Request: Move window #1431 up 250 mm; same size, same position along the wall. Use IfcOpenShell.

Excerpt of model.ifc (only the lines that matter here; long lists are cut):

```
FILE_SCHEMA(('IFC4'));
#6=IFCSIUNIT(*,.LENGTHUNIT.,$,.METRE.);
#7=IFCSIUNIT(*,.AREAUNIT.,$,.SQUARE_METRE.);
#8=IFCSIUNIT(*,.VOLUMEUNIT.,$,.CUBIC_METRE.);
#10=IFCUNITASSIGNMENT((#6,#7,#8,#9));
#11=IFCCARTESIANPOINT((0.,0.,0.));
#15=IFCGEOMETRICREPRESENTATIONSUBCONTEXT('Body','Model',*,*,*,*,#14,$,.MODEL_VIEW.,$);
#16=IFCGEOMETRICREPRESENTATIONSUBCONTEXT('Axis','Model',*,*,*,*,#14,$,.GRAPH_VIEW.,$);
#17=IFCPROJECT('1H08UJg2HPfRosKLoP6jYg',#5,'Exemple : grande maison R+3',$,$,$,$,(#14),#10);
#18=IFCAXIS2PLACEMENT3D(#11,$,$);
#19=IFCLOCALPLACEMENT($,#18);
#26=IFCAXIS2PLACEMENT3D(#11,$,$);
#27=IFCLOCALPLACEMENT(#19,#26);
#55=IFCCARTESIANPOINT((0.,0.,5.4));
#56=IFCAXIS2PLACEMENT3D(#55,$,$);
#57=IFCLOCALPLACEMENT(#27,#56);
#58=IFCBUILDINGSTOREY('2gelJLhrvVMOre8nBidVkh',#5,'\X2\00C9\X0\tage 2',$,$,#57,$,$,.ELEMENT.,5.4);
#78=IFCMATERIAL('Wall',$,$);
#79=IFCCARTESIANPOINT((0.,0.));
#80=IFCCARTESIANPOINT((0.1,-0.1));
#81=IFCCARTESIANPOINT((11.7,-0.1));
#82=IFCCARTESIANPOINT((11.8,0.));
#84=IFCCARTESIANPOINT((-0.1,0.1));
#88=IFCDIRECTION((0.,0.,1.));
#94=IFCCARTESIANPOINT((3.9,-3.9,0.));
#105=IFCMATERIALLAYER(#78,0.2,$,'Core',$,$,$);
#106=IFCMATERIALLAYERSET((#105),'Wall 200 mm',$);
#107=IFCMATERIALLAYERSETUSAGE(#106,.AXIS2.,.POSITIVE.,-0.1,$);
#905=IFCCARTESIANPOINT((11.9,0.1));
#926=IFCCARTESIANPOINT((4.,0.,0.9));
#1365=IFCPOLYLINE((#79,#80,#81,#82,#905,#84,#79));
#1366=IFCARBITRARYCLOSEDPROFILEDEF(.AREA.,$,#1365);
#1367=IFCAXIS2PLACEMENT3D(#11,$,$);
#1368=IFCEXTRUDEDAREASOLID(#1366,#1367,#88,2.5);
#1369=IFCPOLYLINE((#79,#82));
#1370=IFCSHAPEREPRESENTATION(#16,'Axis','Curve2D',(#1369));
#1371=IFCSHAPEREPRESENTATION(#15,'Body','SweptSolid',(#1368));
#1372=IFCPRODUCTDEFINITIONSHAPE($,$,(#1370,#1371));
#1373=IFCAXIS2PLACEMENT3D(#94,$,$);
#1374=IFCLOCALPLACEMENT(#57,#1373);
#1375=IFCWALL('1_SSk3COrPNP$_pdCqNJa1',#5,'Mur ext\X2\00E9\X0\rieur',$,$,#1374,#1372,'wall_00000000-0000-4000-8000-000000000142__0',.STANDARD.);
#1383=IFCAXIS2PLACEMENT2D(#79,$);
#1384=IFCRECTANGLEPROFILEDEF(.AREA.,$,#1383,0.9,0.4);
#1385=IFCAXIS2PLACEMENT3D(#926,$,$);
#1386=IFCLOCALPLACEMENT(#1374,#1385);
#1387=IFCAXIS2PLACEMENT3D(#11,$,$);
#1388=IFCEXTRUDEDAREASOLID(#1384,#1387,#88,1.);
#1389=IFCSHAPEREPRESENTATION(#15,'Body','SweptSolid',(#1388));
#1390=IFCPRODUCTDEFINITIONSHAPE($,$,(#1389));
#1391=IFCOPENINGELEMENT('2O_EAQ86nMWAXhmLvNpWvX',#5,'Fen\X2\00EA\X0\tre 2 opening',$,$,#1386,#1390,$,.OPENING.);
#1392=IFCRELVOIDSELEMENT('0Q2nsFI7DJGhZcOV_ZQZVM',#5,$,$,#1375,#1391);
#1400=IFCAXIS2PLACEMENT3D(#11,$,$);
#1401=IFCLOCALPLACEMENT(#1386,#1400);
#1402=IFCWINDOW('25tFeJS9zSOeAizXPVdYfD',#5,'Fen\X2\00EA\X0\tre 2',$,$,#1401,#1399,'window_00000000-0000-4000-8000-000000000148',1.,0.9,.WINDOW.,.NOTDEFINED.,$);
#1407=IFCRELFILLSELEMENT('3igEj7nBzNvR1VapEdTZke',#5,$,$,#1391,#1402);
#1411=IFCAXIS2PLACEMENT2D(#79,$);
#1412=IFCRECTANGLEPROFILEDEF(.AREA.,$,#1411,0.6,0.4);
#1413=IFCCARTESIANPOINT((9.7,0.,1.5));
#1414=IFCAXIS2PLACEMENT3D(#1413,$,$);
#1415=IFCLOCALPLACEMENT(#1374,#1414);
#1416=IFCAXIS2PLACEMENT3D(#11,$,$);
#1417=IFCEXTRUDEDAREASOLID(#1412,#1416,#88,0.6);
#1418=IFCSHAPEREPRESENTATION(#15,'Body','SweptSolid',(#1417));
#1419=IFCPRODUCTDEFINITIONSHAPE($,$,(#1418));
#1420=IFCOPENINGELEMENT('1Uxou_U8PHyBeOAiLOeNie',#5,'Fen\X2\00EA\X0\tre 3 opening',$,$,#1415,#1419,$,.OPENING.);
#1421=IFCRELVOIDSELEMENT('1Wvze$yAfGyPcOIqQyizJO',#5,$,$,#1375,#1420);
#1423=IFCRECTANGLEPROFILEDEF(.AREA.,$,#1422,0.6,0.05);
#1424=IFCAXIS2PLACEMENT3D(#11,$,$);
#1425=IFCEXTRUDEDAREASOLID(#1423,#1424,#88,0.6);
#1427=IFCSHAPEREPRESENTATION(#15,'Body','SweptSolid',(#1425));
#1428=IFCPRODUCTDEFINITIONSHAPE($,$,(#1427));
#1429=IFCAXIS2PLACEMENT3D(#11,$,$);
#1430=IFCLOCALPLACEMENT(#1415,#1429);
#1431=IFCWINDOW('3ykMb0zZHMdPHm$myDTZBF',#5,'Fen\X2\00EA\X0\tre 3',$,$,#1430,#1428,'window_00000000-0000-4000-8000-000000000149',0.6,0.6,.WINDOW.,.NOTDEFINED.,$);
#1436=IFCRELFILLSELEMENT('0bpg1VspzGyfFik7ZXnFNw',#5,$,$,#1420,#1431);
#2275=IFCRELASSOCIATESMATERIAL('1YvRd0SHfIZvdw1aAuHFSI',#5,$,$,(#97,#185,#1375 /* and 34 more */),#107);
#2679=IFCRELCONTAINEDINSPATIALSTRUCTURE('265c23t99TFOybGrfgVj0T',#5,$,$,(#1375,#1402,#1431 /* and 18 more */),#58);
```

```python
import numpy as np
import ifcopenshell
import ifcopenshell.api.geometry
import ifcopenshell.util.placement
import ifcopenshell.util.unit

model = ifcopenshell.open("model.ifc")
unit_scale = ifcopenshell.util.unit.calculate_unit_scale(model)

window = model.by_guid("3ykMb0zZHMdPHm$myDTZBF")
opening = window.FillsVoids[0].RelatingOpeningElement
dz = 0.25 / unit_scale

shift = np.array([0.0, 0.0, dz])
# The window is placed relative to its opening, so it follows when the opening moves.
matrix = ifcopenshell.util.placement.get_local_placement(opening.ObjectPlacement)
matrix[:3, 3] += shift
ifcopenshell.api.geometry.edit_object_placement(
    model, product=opening, matrix=matrix, is_si=False, should_transform_children=True
)

print(f"moved by {dz * unit_scale:+.3f} m")

model.write("model_rev.ifc")
```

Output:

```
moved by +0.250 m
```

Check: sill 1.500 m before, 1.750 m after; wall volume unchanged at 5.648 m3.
